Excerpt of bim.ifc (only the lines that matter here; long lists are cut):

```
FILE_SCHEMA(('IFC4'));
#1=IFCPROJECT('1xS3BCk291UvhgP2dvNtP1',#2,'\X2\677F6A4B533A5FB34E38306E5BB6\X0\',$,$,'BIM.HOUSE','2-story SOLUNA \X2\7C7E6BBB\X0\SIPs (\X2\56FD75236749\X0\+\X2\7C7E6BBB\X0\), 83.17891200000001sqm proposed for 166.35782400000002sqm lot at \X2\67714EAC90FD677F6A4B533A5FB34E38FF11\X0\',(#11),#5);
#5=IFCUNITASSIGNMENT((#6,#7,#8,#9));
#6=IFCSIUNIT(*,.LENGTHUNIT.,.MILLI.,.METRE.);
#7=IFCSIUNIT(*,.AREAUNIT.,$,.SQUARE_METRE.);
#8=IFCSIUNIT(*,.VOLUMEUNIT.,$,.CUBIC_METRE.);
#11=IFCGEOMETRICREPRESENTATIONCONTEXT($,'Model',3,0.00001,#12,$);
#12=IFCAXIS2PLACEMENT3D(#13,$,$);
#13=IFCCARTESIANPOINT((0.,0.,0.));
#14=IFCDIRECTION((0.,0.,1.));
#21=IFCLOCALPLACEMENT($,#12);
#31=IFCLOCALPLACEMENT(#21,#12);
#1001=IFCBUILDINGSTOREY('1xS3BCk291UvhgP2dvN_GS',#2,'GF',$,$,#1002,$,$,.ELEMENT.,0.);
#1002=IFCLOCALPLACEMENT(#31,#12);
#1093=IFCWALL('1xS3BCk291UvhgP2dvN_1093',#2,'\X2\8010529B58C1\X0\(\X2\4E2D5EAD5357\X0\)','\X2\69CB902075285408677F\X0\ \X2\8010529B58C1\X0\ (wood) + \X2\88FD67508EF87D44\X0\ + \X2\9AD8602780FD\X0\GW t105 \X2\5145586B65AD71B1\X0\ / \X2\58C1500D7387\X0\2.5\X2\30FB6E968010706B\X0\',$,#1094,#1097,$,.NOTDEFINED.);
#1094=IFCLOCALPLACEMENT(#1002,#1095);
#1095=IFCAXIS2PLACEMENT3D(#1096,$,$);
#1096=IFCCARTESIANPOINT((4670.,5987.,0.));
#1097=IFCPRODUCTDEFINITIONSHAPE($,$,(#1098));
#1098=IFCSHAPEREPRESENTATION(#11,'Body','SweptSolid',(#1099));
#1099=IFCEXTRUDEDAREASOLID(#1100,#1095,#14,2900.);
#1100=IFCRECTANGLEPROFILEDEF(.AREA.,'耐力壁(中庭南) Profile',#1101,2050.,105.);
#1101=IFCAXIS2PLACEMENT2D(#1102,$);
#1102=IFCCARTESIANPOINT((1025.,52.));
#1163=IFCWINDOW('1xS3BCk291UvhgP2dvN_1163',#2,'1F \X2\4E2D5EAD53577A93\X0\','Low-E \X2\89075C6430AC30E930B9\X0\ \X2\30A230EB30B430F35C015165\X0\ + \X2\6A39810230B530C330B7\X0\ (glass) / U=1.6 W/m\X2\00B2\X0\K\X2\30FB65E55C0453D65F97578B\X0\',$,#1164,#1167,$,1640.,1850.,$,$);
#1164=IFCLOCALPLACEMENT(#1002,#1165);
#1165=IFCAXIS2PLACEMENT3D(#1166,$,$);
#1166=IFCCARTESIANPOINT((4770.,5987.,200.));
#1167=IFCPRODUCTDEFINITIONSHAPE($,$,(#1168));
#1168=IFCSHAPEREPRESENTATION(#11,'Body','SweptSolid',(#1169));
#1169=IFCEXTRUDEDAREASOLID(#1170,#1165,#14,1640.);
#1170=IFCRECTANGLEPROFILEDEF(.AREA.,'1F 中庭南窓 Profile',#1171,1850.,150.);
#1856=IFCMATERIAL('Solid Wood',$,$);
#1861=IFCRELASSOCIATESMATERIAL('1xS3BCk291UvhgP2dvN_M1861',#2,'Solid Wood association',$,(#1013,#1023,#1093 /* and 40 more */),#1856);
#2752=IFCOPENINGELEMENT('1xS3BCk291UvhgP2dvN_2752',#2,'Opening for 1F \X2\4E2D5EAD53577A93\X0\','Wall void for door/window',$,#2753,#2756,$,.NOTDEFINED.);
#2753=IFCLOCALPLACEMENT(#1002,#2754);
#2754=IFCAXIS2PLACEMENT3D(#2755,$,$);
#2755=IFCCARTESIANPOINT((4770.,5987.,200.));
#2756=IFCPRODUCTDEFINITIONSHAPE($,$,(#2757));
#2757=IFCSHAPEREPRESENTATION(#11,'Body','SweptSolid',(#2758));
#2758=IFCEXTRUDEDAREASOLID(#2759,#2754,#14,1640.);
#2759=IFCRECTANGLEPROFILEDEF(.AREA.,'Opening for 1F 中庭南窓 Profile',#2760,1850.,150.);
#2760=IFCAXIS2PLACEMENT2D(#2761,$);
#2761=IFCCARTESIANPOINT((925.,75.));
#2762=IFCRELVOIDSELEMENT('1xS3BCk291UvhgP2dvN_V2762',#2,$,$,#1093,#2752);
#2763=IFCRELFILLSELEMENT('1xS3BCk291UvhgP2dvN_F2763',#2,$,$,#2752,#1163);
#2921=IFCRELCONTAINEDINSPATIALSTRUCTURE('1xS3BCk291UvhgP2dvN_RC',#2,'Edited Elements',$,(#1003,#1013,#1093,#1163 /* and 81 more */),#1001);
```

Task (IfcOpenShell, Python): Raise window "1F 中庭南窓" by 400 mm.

```python
import numpy as np
import ifcopenshell
import ifcopenshell.api.geometry
import ifcopenshell.util.placement
import ifcopenshell.util.unit

model = ifcopenshell.open("bim.ifc")
unit_scale = ifcopenshell.util.unit.calculate_unit_scale(model)

window = model.by_guid("1xS3BCk291UvhgP2dvN_1163")
opening = window.FillsVoids[0].RelatingOpeningElement
dz = 0.4 / unit_scale

shift = np.array([0.0, 0.0, dz])
# The window is not placed relative to its opening, so move both.
for product in (opening, window):
    matrix = ifcopenshell.util.placement.get_local_placement(product.ObjectPlacement)
    matrix[:3, 3] += shift
    ifcopenshell.api.geometry.edit_object_placement(model, product=product, matrix=matrix, is_si=False)

print(f"moved by {dz * unit_scale:+.3f} m")

model.write("bim_rev.ifc")
```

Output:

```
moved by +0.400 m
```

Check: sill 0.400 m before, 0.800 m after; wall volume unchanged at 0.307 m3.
